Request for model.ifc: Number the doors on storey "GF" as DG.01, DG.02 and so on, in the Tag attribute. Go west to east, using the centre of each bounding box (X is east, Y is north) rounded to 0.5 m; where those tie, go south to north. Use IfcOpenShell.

First a look at what the model holds.

```python
import ifcopenshell
import ifcopenshell.util.element
import ifcopenshell.util.placement

model = ifcopenshell.open("model.ifc")
print(model.schema)
storey = next(s for s in model.by_type("IfcBuildingStorey") if s.Name == "GF")
doors = [e for e in ifcopenshell.util.element.get_decomposition(storey) if e.is_a("IfcDoor")]
for e in sorted(doors, key=lambda e: e.id()):
    origin = ifcopenshell.util.placement.get_local_placement(e.ObjectPlacement)[:3, 3]
    print(e.id(), e.Tag, e.Name, origin.round(2) + 0.0, sep=" | ")
```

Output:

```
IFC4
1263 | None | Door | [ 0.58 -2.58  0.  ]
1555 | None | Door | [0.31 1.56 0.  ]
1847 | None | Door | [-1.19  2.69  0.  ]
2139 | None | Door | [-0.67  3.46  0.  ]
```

```python
import ifcopenshell
import ifcopenshell.geom
import ifcopenshell.util.element
import ifcopenshell.util.shape

model = ifcopenshell.open("model.ifc")
settings = ifcopenshell.geom.settings()
settings.set("use-world-coords", True)


def centre(element):
    shape = ifcopenshell.geom.create_shape(settings, element)
    return ifcopenshell.util.shape.get_bbox_centroid(shape.geometry)


storey = next(s for s in model.by_type("IfcBuildingStorey") if s.Name == "GF")
doors = [e for e in ifcopenshell.util.element.get_decomposition(storey) if e.is_a("IfcDoor")]

# Insertion points can sit at a corner or the storey origin, so sort by the geometry (in metres).
centres = {e: centre(e) for e in doors}
doors.sort(key=lambda e: (round(centres[e][0] / 0.5), centres[e][1]))

for i, e in enumerate(doors, start=1):
    number = f"DG.{i:02d}"
    e.Tag = number
    print(e.id(), number)

model.write("model_v2.ifc")
```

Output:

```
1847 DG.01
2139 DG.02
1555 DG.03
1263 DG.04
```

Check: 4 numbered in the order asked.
